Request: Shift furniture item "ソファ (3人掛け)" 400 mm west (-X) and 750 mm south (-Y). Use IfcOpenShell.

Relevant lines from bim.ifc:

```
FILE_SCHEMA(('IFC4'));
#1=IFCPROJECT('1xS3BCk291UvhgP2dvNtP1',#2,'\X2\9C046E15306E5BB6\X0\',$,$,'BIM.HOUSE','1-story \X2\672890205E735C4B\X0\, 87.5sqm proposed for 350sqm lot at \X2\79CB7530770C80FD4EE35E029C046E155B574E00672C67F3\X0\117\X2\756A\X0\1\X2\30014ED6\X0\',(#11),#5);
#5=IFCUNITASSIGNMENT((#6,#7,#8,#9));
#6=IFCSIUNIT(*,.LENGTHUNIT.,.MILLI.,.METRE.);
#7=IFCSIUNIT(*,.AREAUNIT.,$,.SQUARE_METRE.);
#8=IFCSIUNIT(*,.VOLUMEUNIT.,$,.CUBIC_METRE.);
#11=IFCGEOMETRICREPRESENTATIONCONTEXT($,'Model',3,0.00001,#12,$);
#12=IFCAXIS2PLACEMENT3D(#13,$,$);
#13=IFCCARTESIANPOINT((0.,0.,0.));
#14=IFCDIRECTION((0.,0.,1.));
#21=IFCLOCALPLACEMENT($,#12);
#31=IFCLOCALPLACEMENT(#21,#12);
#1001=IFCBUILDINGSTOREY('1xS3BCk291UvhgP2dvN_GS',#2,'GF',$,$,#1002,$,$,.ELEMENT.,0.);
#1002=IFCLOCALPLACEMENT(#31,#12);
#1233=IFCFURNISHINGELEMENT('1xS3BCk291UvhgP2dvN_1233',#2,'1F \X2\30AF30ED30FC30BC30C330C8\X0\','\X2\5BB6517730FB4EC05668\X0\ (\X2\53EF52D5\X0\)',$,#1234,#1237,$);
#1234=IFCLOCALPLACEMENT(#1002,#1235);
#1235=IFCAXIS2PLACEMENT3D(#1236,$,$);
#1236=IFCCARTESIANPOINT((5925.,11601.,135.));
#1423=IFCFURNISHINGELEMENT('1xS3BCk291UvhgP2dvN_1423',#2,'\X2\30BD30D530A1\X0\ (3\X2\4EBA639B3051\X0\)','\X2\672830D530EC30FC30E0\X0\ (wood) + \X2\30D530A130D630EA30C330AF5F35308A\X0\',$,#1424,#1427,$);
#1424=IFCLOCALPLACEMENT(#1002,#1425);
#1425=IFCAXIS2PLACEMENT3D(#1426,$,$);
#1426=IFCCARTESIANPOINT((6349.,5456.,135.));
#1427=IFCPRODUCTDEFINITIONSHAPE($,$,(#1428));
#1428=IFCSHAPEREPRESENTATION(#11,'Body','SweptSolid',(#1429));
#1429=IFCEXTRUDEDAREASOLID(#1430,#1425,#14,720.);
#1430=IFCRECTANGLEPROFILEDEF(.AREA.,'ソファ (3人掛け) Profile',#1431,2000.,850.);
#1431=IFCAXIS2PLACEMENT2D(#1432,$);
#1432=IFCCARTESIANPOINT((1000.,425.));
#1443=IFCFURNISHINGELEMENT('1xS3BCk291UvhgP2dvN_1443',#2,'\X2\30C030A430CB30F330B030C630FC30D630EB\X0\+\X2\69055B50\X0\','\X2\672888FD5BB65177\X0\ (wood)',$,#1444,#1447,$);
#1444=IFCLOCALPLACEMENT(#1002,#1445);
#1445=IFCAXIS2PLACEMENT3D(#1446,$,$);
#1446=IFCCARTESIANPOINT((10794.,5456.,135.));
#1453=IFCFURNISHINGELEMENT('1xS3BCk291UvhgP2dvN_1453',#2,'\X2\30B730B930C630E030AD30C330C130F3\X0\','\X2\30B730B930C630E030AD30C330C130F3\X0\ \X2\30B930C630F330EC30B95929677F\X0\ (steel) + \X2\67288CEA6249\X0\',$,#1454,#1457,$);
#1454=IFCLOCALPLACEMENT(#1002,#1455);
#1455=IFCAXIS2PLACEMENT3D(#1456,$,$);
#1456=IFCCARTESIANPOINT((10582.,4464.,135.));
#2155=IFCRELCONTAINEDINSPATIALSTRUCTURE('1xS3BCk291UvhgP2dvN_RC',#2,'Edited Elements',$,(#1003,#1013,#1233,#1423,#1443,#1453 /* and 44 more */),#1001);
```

```python
import ifcopenshell
import ifcopenshell.api.geometry
import ifcopenshell.util.placement
import ifcopenshell.util.unit

model = ifcopenshell.open("bim.ifc")
unit_scale = ifcopenshell.util.unit.calculate_unit_scale(model)

item = model.by_guid("1xS3BCk291UvhgP2dvN_1423")
matrix = ifcopenshell.util.placement.get_local_placement(item.ObjectPlacement)
matrix[0, 3] -= 0.4 / unit_scale
matrix[1, 3] -= 0.75 / unit_scale
ifcopenshell.api.geometry.edit_object_placement(model, product=item, matrix=matrix, is_si=False)

print(ifcopenshell.util.placement.get_local_placement(item.ObjectPlacement).round(3) + 0.0)

model.write("bim_edited.ifc")
```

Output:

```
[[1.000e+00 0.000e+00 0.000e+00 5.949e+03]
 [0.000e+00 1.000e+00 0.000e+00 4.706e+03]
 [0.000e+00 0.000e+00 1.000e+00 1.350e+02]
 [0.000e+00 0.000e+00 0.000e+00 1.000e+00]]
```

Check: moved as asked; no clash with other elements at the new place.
